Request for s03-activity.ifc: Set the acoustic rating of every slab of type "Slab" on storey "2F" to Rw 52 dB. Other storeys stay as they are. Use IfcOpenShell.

First a look at what the model holds.

```python
import ifcopenshell
import ifcopenshell.util.element

model = ifcopenshell.open("s03-activity.ifc")
print(model.schema)
storey = next(s for s in model.by_type("IfcBuildingStorey") if s.Name == "2F")
slabs = [e for e in ifcopenshell.util.element.get_decomposition(storey) if e.is_a("IfcSlab")]
seen = {}
for e in slabs:
    element_type = ifcopenshell.util.element.get_type(e)
    key = (element_type.Name if element_type != e and element_type else None, ifcopenshell.util.element.get_pset(e, "Pset_SlabCommon", "AcousticRating"))
    seen[key] = seen.get(key, 0) + 1
for (name, value), count in sorted(seen.items(), key=str):
    print(count, "x", name, "|", value)
```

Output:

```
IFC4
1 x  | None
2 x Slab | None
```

```python
import ifcopenshell
import ifcopenshell.api.pset
import ifcopenshell.util.element

model = ifcopenshell.open("s03-activity.ifc")

storey = next(s for s in model.by_type("IfcBuildingStorey") if s.Name == "2F")
slabs = [e for e in ifcopenshell.util.element.get_decomposition(storey) if e.is_a("IfcSlab")]

count = 0
for e in slabs:
    element_type = ifcopenshell.util.element.get_type(e)
    if element_type in (None, e) or element_type.Name != "Slab":
        continue
    # add_pset returns the element's existing set when there is one.
    pset = ifcopenshell.api.pset.add_pset(model, product=e, name="Pset_SlabCommon")
    ifcopenshell.api.pset.edit_pset(model, pset=pset, properties={"AcousticRating": "Rw 52 dB"})
    count += 1

print(count, "slabs updated")

model.write("s03-activity-out.ifc")
```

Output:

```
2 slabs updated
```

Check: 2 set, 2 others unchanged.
